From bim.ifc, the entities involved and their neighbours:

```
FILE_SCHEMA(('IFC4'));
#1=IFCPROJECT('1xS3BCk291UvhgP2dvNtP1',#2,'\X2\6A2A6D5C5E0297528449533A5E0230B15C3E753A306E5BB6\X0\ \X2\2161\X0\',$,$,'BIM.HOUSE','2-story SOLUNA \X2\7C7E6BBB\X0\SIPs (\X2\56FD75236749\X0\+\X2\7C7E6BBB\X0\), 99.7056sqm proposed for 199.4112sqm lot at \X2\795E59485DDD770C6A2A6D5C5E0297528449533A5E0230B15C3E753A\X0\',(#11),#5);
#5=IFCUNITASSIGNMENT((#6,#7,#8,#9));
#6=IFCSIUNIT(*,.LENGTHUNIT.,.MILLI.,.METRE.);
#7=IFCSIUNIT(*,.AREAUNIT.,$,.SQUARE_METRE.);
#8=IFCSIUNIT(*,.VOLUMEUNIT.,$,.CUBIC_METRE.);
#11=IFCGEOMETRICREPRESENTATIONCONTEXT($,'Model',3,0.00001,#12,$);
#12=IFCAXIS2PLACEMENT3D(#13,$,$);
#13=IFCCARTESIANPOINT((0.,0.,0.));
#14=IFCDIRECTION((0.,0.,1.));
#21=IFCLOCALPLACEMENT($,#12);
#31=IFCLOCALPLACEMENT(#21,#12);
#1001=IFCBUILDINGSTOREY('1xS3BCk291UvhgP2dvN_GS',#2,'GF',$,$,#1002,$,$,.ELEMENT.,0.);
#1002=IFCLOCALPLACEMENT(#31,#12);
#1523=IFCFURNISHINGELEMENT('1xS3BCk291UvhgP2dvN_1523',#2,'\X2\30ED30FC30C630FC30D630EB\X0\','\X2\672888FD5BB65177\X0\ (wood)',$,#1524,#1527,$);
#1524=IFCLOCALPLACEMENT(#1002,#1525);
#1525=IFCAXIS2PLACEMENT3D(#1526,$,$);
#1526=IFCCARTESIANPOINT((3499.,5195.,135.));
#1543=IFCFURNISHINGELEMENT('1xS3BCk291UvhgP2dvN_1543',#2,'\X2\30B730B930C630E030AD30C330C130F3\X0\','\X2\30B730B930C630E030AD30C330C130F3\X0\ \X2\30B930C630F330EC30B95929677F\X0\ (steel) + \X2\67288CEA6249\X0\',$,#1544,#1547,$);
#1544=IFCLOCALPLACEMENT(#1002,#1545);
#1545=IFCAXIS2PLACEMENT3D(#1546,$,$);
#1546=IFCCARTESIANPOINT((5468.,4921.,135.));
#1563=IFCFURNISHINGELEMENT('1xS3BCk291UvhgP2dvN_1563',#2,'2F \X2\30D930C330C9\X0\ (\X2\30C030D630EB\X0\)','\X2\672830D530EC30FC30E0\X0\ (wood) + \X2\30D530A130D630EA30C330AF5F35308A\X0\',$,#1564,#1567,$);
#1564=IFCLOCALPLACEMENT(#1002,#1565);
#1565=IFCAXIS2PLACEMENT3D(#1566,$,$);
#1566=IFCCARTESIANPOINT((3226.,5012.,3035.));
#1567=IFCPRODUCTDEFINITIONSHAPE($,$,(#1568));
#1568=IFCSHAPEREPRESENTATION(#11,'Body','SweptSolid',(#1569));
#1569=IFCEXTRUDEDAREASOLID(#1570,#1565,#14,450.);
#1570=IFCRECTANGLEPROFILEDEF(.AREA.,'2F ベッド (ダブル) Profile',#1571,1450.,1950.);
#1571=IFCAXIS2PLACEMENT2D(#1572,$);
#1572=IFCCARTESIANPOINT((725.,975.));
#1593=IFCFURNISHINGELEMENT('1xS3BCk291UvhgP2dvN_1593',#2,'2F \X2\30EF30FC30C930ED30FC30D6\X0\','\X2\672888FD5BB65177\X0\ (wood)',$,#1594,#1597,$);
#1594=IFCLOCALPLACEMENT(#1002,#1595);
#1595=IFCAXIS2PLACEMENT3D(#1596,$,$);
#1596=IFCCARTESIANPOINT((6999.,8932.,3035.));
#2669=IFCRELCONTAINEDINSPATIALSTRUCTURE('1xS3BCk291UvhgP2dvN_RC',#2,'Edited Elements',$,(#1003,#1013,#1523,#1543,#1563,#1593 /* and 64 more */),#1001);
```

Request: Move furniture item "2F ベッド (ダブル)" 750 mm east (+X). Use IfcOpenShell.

```python
import ifcopenshell
import ifcopenshell.api.geometry
import ifcopenshell.util.placement
import ifcopenshell.util.unit

model = ifcopenshell.open("bim.ifc")
unit_scale = ifcopenshell.util.unit.calculate_unit_scale(model)

item = model.by_id(1563)
matrix = ifcopenshell.util.placement.get_local_placement(item.ObjectPlacement)
matrix[0, 3] += 0.75 / unit_scale
ifcopenshell.api.geometry.edit_object_placement(model, product=item, matrix=matrix, is_si=False)

print(ifcopenshell.util.placement.get_local_placement(item.ObjectPlacement).round(3) + 0.0)

model.write("bim_v2.ifc")
```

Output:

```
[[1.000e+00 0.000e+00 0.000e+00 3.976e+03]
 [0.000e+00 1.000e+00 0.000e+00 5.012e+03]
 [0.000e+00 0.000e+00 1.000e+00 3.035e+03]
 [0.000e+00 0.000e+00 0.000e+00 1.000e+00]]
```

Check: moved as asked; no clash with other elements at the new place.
